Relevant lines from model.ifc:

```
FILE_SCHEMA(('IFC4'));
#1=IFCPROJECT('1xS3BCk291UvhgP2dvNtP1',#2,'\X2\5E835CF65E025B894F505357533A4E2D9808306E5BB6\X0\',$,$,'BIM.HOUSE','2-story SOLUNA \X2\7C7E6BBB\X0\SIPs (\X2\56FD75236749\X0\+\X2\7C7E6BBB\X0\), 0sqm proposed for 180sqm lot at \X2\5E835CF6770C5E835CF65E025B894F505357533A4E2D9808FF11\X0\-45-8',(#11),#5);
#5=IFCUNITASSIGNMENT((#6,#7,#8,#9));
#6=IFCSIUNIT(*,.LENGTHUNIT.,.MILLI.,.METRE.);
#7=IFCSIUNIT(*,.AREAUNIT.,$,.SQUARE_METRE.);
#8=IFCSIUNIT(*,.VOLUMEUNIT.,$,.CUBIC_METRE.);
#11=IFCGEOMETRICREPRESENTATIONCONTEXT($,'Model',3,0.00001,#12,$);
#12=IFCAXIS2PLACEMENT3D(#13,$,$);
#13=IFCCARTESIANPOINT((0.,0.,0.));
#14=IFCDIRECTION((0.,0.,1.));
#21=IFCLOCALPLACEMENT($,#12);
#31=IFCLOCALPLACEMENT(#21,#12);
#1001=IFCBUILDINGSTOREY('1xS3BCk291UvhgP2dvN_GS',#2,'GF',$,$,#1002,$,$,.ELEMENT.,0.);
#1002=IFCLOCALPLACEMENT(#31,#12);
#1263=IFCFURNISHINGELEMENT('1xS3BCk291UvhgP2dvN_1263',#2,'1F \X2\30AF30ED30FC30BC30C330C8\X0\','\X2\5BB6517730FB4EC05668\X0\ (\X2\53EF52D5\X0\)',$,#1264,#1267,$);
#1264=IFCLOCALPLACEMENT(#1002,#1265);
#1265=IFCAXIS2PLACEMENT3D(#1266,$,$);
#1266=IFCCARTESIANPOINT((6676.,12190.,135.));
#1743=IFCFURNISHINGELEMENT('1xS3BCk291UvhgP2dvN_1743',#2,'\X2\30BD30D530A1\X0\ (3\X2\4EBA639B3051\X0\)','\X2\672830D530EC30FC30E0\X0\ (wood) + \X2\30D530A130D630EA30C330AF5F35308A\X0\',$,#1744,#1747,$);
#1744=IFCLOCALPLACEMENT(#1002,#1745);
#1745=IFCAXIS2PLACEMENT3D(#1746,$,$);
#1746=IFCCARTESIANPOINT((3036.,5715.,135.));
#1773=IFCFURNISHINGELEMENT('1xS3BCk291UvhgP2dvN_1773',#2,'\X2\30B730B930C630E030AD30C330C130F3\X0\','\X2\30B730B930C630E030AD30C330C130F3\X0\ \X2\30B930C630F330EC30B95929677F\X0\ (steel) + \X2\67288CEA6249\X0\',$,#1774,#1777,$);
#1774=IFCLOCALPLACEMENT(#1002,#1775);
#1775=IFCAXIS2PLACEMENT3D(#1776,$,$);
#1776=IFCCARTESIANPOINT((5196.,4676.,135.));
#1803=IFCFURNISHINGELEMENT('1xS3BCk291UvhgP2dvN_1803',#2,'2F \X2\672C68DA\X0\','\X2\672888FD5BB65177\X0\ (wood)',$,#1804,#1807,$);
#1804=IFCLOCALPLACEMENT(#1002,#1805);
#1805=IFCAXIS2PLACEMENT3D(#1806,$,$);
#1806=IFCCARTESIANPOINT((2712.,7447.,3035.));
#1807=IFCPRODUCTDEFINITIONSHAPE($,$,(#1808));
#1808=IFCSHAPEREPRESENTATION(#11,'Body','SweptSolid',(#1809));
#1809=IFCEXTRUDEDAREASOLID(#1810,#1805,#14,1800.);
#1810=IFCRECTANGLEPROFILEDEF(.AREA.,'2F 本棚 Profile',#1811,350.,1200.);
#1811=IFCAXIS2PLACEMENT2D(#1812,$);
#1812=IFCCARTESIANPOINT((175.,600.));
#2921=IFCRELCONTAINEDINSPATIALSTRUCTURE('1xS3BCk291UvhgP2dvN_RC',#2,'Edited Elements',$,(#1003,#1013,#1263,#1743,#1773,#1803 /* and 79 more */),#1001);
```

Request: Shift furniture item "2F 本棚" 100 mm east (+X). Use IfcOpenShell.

```python
import ifcopenshell
import ifcopenshell.api.geometry
import ifcopenshell.util.placement
import ifcopenshell.util.unit

model = ifcopenshell.open("model.ifc")
unit_scale = ifcopenshell.util.unit.calculate_unit_scale(model)

item = model.by_guid("1xS3BCk291UvhgP2dvN_1803")
matrix = ifcopenshell.util.placement.get_local_placement(item.ObjectPlacement)
matrix[0, 3] += 0.1 / unit_scale
ifcopenshell.api.geometry.edit_object_placement(model, product=item, matrix=matrix, is_si=False)

print(ifcopenshell.util.placement.get_local_placement(item.ObjectPlacement).round(3) + 0.0)

model.write("model_edited.ifc")
```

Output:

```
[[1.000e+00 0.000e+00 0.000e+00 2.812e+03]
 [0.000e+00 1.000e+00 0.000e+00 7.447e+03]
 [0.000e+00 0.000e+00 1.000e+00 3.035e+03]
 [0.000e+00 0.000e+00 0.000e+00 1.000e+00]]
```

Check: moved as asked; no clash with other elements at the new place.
